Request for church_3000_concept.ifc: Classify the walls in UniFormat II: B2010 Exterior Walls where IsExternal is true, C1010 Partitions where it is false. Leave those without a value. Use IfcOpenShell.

First a look at what the model holds.

```python
import ifcopenshell
import ifcopenshell.util.element

model = ifcopenshell.open("church_3000_concept.ifc")
print(model.schema)
print("classifications:", [c.Name for c in model.by_type("IfcClassification")])
values = [ifcopenshell.util.element.get_pset(e, "Pset_WallCommon", "IsExternal") for e in model.by_type("IfcWall")]
for value in (True, False, None):
    print("IsExternal", value, values.count(value))
```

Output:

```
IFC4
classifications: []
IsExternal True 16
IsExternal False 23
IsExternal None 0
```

```python
import ifcopenshell
import ifcopenshell.api.classification
import ifcopenshell.util.element

model = ifcopenshell.open("church_3000_concept.ifc")

system = ifcopenshell.api.classification.add_classification(model, classification="UniFormat II")

walls = model.by_type("IfcWall")
external = {e: ifcopenshell.util.element.get_pset(e, "Pset_WallCommon", "IsExternal") for e in walls}
for flag, code, name in ((True, "B2010", "Exterior Walls"), (False, "C1010", "Partitions")):
    products = [e for e in walls if external[e] is flag]
    ifcopenshell.api.classification.add_reference(
        model, products=products, classification=system, identification=code, name=name
    )
    print(code, len(products))

model.write("church_3000_concept_updated.ifc")
```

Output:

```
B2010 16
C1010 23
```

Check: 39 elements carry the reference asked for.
